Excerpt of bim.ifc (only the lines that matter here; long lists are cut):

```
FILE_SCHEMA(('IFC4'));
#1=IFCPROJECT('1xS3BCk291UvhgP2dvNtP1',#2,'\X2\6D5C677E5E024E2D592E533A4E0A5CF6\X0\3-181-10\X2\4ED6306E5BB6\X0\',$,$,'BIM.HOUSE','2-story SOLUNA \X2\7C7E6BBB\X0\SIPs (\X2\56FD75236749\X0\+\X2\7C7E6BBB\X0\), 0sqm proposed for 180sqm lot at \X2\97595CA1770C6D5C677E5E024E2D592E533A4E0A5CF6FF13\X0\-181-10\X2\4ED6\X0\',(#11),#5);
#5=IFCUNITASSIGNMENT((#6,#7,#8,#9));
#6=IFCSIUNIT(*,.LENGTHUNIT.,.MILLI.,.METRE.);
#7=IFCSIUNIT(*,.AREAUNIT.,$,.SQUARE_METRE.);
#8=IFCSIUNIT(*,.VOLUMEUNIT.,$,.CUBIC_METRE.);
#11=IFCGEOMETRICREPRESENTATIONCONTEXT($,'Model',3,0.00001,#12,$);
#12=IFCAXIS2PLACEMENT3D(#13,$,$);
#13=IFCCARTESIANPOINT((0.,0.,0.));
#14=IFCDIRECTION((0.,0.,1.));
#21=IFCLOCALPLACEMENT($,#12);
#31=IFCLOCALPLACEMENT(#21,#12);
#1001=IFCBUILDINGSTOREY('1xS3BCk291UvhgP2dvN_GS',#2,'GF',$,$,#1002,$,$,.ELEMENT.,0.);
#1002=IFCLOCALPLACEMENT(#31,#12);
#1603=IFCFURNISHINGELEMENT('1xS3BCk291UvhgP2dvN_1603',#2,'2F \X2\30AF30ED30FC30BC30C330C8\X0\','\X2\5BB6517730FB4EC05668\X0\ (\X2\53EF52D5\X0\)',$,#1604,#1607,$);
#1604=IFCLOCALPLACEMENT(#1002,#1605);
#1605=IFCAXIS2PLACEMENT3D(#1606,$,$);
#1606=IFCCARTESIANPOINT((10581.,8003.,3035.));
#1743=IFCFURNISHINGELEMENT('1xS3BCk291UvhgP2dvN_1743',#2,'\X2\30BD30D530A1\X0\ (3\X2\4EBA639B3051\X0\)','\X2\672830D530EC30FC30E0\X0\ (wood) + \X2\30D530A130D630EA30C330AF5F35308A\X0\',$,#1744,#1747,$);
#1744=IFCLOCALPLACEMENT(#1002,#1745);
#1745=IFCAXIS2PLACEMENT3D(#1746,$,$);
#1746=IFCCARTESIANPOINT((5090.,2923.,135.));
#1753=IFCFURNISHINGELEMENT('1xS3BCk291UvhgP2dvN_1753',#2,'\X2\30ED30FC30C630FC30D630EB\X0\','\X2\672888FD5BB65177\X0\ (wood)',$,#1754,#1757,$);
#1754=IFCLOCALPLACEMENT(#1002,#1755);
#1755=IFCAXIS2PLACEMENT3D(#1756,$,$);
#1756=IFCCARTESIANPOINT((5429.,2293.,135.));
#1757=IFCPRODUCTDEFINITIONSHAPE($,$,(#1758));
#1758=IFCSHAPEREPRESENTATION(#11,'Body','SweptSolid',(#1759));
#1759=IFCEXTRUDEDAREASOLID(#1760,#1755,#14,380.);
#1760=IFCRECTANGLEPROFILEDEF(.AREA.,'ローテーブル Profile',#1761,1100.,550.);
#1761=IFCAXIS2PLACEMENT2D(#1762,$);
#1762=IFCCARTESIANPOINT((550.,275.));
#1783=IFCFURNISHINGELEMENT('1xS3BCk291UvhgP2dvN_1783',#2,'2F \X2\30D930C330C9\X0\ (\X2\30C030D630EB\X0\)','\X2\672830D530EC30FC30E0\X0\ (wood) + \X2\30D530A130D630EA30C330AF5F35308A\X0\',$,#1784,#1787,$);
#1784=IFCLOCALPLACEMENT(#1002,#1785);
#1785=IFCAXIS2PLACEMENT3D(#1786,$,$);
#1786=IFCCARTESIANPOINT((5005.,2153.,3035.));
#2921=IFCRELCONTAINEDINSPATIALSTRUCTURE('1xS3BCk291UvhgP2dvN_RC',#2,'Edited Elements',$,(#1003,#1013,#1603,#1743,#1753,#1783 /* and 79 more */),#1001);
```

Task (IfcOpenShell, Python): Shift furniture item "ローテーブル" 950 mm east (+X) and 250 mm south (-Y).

```python
import ifcopenshell
import ifcopenshell.api.geometry
import ifcopenshell.util.placement

model = ifcopenshell.open("bim.ifc")

item = model.by_guid("1xS3BCk291UvhgP2dvN_1753")
matrix = ifcopenshell.util.placement.get_local_placement(item.ObjectPlacement)
matrix[0, 3] += 950.0
matrix[1, 3] -= 250.0
ifcopenshell.api.geometry.edit_object_placement(model, product=item, matrix=matrix, is_si=False)

print(ifcopenshell.util.placement.get_local_placement(item.ObjectPlacement).round(3) + 0.0)

model.write("bim_rev.ifc")
```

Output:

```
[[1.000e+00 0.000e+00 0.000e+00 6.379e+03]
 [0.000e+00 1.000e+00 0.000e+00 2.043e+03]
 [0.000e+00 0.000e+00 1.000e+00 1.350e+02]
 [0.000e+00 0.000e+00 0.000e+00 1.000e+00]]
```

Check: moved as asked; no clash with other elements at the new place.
